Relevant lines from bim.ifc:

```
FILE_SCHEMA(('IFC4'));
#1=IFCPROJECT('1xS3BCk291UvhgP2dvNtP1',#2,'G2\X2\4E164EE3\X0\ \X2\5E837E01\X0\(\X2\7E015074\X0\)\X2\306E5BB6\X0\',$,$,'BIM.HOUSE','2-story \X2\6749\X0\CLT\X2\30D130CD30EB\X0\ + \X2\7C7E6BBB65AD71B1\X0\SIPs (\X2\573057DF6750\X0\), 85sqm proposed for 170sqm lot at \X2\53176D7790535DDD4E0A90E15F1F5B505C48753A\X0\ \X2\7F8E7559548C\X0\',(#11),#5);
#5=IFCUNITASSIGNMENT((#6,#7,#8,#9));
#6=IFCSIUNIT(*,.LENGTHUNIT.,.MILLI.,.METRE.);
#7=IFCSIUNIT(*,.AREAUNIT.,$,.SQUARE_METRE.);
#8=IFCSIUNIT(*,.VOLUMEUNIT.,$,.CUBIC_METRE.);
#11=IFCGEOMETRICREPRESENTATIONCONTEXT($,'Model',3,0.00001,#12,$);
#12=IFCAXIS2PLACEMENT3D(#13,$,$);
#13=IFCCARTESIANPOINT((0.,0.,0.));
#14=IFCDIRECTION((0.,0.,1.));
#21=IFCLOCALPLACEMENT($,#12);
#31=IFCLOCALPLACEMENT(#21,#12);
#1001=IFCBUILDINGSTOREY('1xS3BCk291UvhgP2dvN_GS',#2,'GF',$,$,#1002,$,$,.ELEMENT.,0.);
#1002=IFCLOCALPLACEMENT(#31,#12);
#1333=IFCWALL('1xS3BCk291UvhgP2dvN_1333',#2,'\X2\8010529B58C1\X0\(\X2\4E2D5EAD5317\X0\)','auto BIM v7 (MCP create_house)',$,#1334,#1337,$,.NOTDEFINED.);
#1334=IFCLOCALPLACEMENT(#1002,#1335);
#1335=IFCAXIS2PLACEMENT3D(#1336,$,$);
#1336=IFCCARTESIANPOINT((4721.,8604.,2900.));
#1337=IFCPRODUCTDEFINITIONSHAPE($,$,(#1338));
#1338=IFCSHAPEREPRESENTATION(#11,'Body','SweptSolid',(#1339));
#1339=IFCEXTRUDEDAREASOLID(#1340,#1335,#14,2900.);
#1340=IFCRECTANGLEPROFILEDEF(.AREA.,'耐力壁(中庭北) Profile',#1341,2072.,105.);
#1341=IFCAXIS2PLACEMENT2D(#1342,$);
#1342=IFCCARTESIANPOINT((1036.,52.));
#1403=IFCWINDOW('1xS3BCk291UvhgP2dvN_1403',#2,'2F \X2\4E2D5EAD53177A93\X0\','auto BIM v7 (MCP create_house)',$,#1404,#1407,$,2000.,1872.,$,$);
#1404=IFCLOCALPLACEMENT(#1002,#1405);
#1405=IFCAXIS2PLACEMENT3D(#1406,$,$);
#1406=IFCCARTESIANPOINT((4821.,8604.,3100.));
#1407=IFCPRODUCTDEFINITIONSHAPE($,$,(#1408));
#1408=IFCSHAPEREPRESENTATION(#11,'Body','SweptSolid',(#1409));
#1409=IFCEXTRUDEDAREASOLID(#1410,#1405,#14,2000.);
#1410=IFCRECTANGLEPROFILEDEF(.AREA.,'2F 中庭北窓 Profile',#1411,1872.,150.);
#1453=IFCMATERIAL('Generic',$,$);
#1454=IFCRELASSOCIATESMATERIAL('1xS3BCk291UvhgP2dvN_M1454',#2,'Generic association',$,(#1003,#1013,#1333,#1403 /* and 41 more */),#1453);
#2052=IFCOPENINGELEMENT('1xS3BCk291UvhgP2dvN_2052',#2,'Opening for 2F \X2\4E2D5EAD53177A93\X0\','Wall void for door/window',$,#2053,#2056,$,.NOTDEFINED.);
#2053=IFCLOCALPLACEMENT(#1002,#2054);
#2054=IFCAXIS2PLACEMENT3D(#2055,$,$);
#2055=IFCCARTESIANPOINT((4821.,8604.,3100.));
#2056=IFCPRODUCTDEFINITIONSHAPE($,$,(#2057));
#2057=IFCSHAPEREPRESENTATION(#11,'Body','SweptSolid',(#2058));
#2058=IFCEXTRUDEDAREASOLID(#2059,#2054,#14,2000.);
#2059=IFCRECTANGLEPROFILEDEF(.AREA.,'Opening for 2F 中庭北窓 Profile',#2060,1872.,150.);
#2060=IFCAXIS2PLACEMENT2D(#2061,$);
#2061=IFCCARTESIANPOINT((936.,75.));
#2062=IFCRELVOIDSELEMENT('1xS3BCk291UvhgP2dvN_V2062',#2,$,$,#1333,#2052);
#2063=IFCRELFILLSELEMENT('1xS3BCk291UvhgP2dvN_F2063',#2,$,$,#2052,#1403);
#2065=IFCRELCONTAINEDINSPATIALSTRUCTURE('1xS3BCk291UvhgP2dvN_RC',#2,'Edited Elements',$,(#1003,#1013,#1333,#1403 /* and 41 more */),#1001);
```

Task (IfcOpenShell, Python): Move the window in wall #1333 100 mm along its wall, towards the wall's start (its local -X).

```python
import ifcopenshell
import ifcopenshell.api.geometry
import ifcopenshell.util.placement
import ifcopenshell.util.unit

model = ifcopenshell.open("bim.ifc")
unit_scale = ifcopenshell.util.unit.calculate_unit_scale(model)

window = model.by_guid("1xS3BCk291UvhgP2dvN_1403")
opening = window.FillsVoids[0].RelatingOpeningElement
wall = opening.VoidsElements[0].RelatingBuildingElement

wall_matrix = ifcopenshell.util.placement.get_local_placement(wall.ObjectPlacement)
shift = wall_matrix[:3, 0] * -0.1 / unit_scale
before = ifcopenshell.util.placement.get_local_placement(window.ObjectPlacement)[:3, 3].copy()

# The window is not placed relative to its opening, so move both.
for product in (opening, window):
    matrix = ifcopenshell.util.placement.get_local_placement(product.ObjectPlacement)
    matrix[:3, 3] += shift
    ifcopenshell.api.geometry.edit_object_placement(model, product=product, matrix=matrix, is_si=False)

after = ifcopenshell.util.placement.get_local_placement(window.ObjectPlacement)[:3, 3]
print("window moved by", (after - before).round(3) + 0.0)

model.write("bim_rev.ifc")
```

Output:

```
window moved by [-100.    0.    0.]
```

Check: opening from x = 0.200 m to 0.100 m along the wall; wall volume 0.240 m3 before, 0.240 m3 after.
